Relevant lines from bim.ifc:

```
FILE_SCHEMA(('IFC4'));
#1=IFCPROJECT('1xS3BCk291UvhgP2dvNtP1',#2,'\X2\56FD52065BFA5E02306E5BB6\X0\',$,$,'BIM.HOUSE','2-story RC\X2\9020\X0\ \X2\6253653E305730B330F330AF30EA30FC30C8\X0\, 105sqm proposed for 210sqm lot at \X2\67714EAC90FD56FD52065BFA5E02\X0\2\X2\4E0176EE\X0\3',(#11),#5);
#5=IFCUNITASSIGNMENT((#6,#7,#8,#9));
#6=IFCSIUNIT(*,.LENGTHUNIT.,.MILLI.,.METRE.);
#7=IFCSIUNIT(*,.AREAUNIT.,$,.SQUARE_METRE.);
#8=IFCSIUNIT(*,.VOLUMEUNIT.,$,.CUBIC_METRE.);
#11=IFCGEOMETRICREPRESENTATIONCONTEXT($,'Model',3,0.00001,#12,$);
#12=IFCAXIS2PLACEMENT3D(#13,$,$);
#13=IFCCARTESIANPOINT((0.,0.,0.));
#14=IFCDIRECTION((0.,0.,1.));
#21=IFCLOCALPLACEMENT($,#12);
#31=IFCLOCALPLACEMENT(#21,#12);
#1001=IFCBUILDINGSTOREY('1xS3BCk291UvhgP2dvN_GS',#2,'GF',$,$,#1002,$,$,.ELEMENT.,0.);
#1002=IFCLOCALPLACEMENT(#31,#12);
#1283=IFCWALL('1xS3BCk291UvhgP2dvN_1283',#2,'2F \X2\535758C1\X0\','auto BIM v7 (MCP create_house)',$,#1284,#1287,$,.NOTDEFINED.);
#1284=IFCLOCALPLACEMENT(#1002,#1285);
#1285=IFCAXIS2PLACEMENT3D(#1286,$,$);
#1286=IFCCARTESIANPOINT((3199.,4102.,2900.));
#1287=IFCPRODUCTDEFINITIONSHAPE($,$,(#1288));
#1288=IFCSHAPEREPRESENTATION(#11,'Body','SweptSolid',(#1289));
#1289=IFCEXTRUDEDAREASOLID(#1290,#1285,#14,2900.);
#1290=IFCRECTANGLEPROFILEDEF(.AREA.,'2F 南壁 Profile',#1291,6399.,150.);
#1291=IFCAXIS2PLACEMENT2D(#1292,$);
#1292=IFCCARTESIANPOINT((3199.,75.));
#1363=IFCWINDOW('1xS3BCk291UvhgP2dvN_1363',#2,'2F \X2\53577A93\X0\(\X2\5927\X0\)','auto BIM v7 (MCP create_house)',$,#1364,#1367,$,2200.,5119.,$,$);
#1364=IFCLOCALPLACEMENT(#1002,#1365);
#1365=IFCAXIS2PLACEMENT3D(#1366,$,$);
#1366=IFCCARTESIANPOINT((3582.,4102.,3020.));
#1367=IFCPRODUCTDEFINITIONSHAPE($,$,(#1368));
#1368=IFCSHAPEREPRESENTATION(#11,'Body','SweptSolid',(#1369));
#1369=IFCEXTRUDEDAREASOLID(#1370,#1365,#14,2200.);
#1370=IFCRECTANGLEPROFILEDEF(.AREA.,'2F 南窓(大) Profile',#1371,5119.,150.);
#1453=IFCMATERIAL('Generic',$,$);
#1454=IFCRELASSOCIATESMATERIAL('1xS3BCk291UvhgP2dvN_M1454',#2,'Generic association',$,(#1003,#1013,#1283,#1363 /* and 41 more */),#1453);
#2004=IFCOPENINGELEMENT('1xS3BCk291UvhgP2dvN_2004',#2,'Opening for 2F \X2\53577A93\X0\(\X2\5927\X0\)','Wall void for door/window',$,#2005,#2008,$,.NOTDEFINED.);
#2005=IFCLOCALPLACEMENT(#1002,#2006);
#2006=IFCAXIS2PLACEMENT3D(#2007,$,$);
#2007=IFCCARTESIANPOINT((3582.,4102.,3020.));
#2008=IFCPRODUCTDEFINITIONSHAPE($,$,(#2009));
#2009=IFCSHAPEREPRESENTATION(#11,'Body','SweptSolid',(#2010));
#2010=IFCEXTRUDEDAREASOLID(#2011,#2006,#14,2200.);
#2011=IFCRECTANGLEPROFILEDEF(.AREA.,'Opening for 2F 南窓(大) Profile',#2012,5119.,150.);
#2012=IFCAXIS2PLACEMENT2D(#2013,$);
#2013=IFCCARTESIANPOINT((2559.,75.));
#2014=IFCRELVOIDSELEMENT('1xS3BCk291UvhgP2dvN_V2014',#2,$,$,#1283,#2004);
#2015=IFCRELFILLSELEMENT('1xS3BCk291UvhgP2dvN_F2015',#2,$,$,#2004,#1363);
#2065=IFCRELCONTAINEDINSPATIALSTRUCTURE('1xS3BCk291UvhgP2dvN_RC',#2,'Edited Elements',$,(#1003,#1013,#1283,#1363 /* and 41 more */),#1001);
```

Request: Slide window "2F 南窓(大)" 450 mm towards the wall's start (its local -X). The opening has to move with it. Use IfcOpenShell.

```python
import ifcopenshell
import ifcopenshell.api.geometry
import ifcopenshell.util.placement
import ifcopenshell.util.unit

model = ifcopenshell.open("bim.ifc")
unit_scale = ifcopenshell.util.unit.calculate_unit_scale(model)

window = model.by_id(1363)
opening = window.FillsVoids[0].RelatingOpeningElement
wall = opening.VoidsElements[0].RelatingBuildingElement

wall_matrix = ifcopenshell.util.placement.get_local_placement(wall.ObjectPlacement)
shift = wall_matrix[:3, 0] * -0.45 / unit_scale
before = ifcopenshell.util.placement.get_local_placement(window.ObjectPlacement)[:3, 3].copy()

# The window is not placed relative to its opening, so move both.
for product in (opening, window):
    matrix = ifcopenshell.util.placement.get_local_placement(product.ObjectPlacement)
    matrix[:3, 3] += shift
    ifcopenshell.api.geometry.edit_object_placement(model, product=product, matrix=matrix, is_si=False)

after = ifcopenshell.util.placement.get_local_placement(window.ObjectPlacement)[:3, 3]
print("window moved by", (after - before).round(3) + 0.0)

model.write("bim_v2.ifc")
```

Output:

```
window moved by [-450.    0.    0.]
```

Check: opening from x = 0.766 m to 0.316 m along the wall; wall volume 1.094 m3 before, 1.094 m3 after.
